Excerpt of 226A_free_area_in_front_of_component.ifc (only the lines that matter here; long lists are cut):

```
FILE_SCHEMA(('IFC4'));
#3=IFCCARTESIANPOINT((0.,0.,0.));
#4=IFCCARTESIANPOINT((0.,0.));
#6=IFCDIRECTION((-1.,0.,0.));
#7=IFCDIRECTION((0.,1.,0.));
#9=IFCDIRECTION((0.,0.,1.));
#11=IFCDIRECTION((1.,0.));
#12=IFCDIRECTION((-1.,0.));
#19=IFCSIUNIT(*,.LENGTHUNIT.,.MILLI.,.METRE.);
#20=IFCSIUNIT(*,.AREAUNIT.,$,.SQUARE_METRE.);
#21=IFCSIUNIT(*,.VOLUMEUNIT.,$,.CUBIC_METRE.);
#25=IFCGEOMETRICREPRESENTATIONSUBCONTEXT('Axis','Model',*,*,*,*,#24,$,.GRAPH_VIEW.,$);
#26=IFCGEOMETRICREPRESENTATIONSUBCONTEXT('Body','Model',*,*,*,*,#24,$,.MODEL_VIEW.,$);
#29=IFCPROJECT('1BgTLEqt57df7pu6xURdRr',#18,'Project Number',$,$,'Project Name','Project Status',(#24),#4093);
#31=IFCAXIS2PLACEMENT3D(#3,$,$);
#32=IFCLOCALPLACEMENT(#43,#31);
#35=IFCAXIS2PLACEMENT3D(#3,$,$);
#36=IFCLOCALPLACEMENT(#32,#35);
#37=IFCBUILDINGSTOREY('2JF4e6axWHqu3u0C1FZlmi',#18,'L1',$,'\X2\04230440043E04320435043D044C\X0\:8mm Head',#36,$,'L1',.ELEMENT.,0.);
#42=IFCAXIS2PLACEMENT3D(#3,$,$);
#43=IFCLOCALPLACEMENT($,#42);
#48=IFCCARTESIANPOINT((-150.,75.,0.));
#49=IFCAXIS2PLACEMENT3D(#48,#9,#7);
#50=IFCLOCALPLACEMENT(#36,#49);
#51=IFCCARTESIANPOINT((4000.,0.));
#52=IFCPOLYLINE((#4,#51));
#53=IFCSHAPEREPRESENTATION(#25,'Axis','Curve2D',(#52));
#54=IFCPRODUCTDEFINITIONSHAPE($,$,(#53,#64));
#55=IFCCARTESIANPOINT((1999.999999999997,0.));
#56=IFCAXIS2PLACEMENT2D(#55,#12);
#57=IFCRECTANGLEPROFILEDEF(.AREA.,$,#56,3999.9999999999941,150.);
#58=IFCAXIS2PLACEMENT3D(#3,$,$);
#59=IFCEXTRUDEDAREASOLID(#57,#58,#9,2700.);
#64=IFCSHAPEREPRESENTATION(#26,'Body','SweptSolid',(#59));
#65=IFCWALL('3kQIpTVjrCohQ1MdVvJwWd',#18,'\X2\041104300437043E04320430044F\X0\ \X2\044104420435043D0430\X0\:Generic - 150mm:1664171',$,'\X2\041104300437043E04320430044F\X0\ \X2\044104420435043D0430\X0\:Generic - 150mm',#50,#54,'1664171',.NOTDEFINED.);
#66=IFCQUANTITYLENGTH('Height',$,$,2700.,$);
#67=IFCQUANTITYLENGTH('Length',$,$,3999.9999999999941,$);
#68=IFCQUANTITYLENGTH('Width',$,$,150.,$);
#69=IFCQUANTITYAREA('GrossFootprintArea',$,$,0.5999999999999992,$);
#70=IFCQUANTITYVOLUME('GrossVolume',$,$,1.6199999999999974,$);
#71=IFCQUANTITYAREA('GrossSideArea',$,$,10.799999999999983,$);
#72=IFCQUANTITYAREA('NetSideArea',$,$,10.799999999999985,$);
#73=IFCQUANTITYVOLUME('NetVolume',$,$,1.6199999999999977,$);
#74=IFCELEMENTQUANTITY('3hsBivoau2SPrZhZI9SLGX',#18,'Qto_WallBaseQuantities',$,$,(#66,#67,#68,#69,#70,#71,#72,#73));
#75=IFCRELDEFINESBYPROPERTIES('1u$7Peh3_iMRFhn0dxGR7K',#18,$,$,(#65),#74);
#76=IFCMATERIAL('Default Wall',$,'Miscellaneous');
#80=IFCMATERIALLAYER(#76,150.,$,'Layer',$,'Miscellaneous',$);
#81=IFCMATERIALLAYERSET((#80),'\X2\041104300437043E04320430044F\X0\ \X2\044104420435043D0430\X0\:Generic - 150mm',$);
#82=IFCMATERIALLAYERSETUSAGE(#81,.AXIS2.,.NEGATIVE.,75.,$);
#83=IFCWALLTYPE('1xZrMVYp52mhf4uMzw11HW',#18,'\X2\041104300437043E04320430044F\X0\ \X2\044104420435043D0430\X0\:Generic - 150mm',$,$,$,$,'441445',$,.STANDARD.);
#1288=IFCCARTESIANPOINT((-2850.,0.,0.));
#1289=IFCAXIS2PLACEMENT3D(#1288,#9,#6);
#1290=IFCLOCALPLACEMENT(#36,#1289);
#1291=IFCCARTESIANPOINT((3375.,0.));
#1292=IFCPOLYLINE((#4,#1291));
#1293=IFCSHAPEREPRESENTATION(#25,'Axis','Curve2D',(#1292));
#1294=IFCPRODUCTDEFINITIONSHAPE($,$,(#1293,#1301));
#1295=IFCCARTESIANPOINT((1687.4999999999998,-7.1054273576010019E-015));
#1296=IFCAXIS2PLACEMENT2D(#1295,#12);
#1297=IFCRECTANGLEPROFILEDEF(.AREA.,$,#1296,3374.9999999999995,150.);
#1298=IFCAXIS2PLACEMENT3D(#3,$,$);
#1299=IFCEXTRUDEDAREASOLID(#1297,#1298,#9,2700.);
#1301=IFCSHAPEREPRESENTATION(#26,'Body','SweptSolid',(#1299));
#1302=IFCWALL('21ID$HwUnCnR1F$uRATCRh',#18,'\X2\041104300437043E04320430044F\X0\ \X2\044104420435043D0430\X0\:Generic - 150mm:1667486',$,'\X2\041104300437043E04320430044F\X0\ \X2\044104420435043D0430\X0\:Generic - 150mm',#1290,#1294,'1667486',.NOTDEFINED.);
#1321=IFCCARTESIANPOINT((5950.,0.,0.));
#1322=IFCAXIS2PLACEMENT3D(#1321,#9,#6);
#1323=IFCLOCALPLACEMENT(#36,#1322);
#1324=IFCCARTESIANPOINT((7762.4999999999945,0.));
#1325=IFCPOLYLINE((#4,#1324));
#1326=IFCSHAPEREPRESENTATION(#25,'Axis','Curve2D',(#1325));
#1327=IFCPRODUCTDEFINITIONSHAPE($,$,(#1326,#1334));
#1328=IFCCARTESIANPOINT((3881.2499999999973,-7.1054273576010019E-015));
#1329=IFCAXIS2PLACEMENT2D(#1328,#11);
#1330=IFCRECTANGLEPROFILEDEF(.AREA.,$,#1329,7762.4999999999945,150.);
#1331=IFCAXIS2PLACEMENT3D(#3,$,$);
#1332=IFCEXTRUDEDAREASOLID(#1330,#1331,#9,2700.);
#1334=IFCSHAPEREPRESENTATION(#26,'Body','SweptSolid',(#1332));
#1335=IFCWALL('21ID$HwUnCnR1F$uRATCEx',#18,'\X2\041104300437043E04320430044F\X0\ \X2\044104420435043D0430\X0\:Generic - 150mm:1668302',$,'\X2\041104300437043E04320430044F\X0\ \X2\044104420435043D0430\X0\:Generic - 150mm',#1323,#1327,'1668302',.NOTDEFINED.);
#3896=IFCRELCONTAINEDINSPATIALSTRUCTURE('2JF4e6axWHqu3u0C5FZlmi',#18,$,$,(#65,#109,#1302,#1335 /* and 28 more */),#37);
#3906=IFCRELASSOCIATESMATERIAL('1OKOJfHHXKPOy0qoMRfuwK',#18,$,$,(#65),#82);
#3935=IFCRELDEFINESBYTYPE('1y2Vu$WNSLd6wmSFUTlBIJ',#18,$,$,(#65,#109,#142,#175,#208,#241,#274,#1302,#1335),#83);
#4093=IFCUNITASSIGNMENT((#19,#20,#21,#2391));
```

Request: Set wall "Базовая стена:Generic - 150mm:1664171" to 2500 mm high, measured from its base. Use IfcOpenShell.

```python
import ifcopenshell
import ifcopenshell.api.pset
import ifcopenshell.geom
import ifcopenshell.util.element
import ifcopenshell.util.representation
import ifcopenshell.util.shape
import ifcopenshell.util.unit

model = ifcopenshell.open("226A_free_area_in_front_of_component.ifc")
unit_scale = ifcopenshell.util.unit.calculate_unit_scale(model)
area_scale = ifcopenshell.util.unit.calculate_unit_scale(model, "AREAUNIT")
volume_scale = ifcopenshell.util.unit.calculate_unit_scale(model, "VOLUMEUNIT")
settings = ifcopenshell.geom.settings()


def volume(element):
    """Net volume in cubic metres, openings subtracted."""
    shape = ifcopenshell.geom.create_shape(settings, element)
    return ifcopenshell.util.shape.get_volume(shape.geometry)


wall = model.by_guid("3kQIpTVjrCohQ1MdVvJwWd")
before = volume(wall)

body = ifcopenshell.util.representation.get_representation(wall, "Model", "Body")
solid = body.Items[0]
old_height = solid.Depth
solid.Depth = 2500.0
after = volume(wall)
thickness = 0.15  # wall thickness in metres

# Update the stored height, areas and volumes.
qto = model.by_id(ifcopenshell.util.element.get_pset(wall, "Qto_WallBaseQuantities", should_inherit=False)["id"])
ifcopenshell.api.pset.edit_qto(model, qto=qto, properties={
    "Height": solid.Depth,
    "GrossVolume": ifcopenshell.util.element.get_pset(wall, "Qto_WallBaseQuantities", "GrossVolume") * solid.Depth / old_height,
    "GrossSideArea": ifcopenshell.util.element.get_pset(wall, "Qto_WallBaseQuantities", "GrossSideArea") * solid.Depth / old_height,
    "NetSideArea": after / thickness / area_scale,
    "NetVolume": after / volume_scale,
})

print(f"height {old_height:g} -> {solid.Depth:g}, volume {before:.3f} -> {after:.3f} m3")

model.write("226A_free_area_in_front_of_component_rev.ifc")
```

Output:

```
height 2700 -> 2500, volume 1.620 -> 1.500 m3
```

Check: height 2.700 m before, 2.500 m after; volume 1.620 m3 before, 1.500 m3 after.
